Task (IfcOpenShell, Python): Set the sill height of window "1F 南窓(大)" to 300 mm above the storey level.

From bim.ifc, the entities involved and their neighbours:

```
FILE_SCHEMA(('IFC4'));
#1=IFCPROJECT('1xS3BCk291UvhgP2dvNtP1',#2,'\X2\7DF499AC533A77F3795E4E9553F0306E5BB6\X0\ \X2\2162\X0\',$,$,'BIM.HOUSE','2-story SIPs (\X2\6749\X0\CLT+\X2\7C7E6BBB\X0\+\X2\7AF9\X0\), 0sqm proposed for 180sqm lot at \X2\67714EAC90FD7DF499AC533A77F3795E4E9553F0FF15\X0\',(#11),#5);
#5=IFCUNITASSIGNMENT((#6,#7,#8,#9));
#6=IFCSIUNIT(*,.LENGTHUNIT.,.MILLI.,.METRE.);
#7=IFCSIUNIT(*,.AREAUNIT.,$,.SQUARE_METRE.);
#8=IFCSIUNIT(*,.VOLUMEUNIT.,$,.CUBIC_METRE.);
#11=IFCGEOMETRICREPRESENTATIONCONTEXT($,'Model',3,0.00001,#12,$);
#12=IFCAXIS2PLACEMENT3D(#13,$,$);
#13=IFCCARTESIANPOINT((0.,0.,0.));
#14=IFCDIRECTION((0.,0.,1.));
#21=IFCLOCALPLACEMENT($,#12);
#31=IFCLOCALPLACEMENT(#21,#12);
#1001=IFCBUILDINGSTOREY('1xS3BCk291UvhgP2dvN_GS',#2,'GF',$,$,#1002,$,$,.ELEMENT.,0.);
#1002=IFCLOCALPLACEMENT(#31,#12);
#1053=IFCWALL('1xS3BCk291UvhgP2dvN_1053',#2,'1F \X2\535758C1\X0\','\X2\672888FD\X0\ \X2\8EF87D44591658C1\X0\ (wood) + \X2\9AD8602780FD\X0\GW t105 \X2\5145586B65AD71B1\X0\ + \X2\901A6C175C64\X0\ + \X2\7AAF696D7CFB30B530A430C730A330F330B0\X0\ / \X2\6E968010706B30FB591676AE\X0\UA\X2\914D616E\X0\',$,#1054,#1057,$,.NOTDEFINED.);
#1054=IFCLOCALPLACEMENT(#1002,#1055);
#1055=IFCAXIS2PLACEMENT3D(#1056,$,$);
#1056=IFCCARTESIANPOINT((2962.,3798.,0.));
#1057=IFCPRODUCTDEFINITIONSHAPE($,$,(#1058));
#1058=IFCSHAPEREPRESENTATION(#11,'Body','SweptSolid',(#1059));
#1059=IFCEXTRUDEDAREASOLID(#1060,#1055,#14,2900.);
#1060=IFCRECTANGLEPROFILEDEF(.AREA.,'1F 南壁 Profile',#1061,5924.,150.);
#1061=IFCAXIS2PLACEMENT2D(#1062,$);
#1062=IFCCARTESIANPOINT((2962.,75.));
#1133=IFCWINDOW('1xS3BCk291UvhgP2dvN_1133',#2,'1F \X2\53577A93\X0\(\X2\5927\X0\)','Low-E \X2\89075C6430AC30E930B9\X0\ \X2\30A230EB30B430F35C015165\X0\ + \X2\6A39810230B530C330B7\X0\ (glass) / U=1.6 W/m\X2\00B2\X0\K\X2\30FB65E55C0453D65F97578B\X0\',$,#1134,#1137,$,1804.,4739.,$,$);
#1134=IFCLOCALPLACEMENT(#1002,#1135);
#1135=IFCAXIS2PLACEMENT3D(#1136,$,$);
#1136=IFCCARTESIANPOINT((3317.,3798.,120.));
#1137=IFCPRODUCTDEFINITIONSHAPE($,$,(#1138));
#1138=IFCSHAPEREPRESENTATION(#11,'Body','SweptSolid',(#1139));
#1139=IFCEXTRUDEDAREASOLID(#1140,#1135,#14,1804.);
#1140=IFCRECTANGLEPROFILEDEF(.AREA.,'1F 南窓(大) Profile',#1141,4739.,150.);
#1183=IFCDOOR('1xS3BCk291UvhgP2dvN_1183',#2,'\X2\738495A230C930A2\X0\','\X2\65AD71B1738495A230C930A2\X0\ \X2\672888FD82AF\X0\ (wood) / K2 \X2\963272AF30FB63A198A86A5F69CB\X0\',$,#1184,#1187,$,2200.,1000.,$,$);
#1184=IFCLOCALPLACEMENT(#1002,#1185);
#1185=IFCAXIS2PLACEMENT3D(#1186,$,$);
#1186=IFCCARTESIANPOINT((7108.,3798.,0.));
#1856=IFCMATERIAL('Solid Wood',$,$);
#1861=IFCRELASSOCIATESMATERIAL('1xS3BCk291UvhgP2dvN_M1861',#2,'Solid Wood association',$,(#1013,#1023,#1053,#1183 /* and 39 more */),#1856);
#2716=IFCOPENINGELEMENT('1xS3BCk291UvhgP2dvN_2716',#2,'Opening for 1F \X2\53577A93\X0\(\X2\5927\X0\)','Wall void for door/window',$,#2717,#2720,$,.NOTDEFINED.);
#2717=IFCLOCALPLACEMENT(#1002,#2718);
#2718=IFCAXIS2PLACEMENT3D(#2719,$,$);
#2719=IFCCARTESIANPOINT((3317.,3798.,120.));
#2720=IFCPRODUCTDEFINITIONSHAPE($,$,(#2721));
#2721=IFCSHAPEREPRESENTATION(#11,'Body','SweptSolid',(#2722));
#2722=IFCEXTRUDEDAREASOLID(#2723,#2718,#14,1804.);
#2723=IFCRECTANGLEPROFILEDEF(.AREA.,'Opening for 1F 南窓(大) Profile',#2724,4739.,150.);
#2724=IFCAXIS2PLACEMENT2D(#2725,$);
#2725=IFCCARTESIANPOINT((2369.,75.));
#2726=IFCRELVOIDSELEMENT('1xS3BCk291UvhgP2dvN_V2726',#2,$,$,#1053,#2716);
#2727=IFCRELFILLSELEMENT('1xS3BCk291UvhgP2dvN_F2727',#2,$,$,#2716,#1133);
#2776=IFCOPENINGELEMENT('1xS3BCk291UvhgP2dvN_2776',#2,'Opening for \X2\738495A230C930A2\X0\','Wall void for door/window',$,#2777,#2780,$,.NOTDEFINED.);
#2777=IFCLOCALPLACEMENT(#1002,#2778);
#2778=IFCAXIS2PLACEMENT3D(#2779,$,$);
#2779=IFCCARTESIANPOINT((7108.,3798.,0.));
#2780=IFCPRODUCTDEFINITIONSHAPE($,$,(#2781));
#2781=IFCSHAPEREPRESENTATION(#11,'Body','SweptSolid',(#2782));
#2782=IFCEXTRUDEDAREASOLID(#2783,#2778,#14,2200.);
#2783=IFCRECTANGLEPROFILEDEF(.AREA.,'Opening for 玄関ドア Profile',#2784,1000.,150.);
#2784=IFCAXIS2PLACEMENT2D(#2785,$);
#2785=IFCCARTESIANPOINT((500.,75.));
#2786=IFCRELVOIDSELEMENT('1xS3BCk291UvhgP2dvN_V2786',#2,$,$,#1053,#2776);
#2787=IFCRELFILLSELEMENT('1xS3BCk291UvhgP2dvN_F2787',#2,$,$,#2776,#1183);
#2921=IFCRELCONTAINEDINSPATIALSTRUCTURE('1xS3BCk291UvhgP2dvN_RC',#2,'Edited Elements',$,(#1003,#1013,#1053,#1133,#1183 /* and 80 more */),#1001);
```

```python
import numpy as np
import ifcopenshell
import ifcopenshell.api.geometry
import ifcopenshell.geom
import ifcopenshell.util.element
import ifcopenshell.util.placement
import ifcopenshell.util.shape
import ifcopenshell.util.unit

model = ifcopenshell.open("bim.ifc")
unit_scale = ifcopenshell.util.unit.calculate_unit_scale(model)

window = model.by_guid("1xS3BCk291UvhgP2dvN_1133")
opening = window.FillsVoids[0].RelatingOpeningElement
storey = ifcopenshell.util.element.get_container(window, ifc_class="IfcBuildingStorey")
level = ifcopenshell.util.placement.get_local_placement(storey.ObjectPlacement)[2, 3]

# The opening's origin need not be at the sill, so measure its lowest point.
shape = ifcopenshell.geom.create_shape(ifcopenshell.geom.settings(), opening)
bottom = ifcopenshell.util.shape.get_shape_bottom_elevation(shape, shape.geometry) / unit_scale
dz = level + 0.3 / unit_scale - bottom

shift = np.array([0.0, 0.0, dz])
# The window is not placed relative to its opening, so move both.
for product in (opening, window):
    matrix = ifcopenshell.util.placement.get_local_placement(product.ObjectPlacement)
    matrix[:3, 3] += shift
    ifcopenshell.api.geometry.edit_object_placement(model, product=product, matrix=matrix, is_si=False)

print(f"moved by {dz * unit_scale:+.3f} m")

model.write("bim_edited.ifc")
```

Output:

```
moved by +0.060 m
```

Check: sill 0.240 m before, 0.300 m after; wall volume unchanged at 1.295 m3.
